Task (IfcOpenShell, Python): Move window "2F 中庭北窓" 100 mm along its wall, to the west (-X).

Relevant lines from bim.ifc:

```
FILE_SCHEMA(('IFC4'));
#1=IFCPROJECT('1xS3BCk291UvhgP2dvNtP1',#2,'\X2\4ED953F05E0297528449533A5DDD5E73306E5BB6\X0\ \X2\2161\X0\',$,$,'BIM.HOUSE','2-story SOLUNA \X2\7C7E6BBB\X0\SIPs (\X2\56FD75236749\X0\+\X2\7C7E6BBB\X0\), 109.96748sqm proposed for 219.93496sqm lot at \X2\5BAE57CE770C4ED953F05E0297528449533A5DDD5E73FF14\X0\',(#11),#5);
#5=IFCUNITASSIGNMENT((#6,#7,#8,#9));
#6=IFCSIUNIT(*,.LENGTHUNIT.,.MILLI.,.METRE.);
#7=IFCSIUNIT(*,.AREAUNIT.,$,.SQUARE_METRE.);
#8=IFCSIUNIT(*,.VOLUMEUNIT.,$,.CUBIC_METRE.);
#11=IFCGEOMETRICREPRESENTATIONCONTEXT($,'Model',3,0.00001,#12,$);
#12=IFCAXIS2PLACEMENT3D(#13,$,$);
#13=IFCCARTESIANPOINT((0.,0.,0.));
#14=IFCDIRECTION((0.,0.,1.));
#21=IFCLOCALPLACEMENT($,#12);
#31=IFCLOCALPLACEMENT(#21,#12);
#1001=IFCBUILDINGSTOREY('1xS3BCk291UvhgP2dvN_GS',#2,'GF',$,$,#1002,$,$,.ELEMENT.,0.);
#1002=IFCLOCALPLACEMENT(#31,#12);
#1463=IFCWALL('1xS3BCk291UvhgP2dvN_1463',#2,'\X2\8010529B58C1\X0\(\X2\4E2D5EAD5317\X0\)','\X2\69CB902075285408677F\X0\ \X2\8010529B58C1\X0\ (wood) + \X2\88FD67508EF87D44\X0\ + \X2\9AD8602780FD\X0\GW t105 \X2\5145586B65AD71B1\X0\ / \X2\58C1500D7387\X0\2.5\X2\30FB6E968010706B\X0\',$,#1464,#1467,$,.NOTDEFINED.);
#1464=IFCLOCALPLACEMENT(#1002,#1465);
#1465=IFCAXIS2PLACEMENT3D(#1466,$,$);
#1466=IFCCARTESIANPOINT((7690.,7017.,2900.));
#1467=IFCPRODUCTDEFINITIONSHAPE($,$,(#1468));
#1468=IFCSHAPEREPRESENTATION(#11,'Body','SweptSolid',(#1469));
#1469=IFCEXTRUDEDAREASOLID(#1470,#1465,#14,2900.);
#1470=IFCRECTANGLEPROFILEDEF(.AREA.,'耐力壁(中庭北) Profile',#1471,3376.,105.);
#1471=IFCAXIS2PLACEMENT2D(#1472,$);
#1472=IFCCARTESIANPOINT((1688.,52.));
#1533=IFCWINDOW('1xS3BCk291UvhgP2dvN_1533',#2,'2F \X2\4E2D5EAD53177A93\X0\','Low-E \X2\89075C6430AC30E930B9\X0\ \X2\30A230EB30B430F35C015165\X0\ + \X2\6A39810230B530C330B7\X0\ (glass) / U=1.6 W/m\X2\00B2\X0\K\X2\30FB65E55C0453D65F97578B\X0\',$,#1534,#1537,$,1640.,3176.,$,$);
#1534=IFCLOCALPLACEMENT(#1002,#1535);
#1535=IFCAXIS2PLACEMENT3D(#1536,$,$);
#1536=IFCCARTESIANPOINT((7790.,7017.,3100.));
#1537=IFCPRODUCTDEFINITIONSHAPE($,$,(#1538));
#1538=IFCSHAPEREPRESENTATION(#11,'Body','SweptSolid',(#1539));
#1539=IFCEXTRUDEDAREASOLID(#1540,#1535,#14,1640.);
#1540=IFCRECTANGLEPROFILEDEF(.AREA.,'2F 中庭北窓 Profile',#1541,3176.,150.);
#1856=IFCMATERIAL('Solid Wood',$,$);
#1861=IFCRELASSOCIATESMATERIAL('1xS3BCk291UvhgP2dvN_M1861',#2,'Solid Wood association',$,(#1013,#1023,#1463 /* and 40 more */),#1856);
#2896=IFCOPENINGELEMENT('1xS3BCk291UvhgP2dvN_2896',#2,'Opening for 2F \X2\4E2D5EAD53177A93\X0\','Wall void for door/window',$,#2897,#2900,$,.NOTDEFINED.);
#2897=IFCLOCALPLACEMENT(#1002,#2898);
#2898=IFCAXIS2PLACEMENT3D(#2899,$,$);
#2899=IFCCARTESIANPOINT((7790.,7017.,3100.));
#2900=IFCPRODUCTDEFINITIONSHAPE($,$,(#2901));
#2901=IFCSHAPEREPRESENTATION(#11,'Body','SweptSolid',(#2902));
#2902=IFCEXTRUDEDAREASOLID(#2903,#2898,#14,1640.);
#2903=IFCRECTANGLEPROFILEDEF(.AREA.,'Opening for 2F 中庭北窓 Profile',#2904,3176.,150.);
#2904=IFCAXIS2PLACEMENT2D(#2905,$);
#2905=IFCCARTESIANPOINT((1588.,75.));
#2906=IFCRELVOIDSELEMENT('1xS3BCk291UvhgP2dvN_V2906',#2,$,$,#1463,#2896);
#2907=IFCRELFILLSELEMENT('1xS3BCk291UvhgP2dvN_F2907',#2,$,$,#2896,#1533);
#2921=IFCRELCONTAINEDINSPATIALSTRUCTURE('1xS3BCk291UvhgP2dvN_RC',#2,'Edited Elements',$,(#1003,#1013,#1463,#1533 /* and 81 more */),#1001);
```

```python
import ifcopenshell
import ifcopenshell.api.geometry
import ifcopenshell.util.placement
import ifcopenshell.util.unit

model = ifcopenshell.open("bim.ifc")
unit_scale = ifcopenshell.util.unit.calculate_unit_scale(model)

window = model.by_guid("1xS3BCk291UvhgP2dvN_1533")
opening = window.FillsVoids[0].RelatingOpeningElement
wall = opening.VoidsElements[0].RelatingBuildingElement

wall_matrix = ifcopenshell.util.placement.get_local_placement(wall.ObjectPlacement)
shift = wall_matrix[:3, 0] * -0.1 / unit_scale
before = ifcopenshell.util.placement.get_local_placement(window.ObjectPlacement)[:3, 3].copy()

# The window is not placed relative to its opening, so move both.
for product in (opening, window):
    matrix = ifcopenshell.util.placement.get_local_placement(product.ObjectPlacement)
    matrix[:3, 3] += shift
    ifcopenshell.api.geometry.edit_object_placement(model, product=product, matrix=matrix, is_si=False)

after = ifcopenshell.util.placement.get_local_placement(window.ObjectPlacement)[:3, 3]
print("window moved by", (after - before).round(3) + 0.0)

model.write("bim_v2.ifc")
```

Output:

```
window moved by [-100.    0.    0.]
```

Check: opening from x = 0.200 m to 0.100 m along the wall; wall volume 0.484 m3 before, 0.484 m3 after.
